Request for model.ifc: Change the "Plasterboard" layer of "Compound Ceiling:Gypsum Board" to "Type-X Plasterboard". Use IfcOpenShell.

First a look at what the model holds.

```python
import ifcopenshell
import ifcopenshell.util.element

model = ifcopenshell.open("model.ifc")
print(model.schema)
for layer_set in model.by_type("IfcMaterialLayerSet"):
    if layer_set.LayerSetName == "Compound Ceiling:Gypsum Board":
        for layer in layer_set.MaterialLayers:
            print(layer.id(), layer.Material and layer.Material.Name, layer.LayerThickness, sep=" | ")
        print(len(ifcopenshell.util.element.get_elements_by_material(model, layer_set)), "elements and types use it")
print(sorted(m.Name for m in model.by_type("IfcMaterial") if m.Name)[:60])
```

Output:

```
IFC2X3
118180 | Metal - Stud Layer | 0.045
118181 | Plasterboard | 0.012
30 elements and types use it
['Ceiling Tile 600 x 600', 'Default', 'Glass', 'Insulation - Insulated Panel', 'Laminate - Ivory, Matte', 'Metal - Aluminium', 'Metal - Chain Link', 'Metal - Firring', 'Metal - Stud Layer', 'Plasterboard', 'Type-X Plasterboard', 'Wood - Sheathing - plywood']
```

```python
import ifcopenshell
import ifcopenshell.api.material

model = ifcopenshell.open("model.ifc")

layer_set = next(s for s in model.by_type("IfcMaterialLayerSet") if s.LayerSetName == "Compound Ceiling:Gypsum Board")
layer = next(l for l in layer_set.MaterialLayers if l.Material and l.Material.Name == "Plasterboard")
material = next(m for m in model.by_type("IfcMaterial") if m.Name == "Type-X Plasterboard")

# Point this one layer at the other material; renaming the old one would change it everywhere.
ifcopenshell.api.material.edit_layer(model, layer=layer, attributes={}, material=material)

print([l.Material.Name if l.Material else None for l in layer_set.MaterialLayers])

model.write("model_rev.ifc")
```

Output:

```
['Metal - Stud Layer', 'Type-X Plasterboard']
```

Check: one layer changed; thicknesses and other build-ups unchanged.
